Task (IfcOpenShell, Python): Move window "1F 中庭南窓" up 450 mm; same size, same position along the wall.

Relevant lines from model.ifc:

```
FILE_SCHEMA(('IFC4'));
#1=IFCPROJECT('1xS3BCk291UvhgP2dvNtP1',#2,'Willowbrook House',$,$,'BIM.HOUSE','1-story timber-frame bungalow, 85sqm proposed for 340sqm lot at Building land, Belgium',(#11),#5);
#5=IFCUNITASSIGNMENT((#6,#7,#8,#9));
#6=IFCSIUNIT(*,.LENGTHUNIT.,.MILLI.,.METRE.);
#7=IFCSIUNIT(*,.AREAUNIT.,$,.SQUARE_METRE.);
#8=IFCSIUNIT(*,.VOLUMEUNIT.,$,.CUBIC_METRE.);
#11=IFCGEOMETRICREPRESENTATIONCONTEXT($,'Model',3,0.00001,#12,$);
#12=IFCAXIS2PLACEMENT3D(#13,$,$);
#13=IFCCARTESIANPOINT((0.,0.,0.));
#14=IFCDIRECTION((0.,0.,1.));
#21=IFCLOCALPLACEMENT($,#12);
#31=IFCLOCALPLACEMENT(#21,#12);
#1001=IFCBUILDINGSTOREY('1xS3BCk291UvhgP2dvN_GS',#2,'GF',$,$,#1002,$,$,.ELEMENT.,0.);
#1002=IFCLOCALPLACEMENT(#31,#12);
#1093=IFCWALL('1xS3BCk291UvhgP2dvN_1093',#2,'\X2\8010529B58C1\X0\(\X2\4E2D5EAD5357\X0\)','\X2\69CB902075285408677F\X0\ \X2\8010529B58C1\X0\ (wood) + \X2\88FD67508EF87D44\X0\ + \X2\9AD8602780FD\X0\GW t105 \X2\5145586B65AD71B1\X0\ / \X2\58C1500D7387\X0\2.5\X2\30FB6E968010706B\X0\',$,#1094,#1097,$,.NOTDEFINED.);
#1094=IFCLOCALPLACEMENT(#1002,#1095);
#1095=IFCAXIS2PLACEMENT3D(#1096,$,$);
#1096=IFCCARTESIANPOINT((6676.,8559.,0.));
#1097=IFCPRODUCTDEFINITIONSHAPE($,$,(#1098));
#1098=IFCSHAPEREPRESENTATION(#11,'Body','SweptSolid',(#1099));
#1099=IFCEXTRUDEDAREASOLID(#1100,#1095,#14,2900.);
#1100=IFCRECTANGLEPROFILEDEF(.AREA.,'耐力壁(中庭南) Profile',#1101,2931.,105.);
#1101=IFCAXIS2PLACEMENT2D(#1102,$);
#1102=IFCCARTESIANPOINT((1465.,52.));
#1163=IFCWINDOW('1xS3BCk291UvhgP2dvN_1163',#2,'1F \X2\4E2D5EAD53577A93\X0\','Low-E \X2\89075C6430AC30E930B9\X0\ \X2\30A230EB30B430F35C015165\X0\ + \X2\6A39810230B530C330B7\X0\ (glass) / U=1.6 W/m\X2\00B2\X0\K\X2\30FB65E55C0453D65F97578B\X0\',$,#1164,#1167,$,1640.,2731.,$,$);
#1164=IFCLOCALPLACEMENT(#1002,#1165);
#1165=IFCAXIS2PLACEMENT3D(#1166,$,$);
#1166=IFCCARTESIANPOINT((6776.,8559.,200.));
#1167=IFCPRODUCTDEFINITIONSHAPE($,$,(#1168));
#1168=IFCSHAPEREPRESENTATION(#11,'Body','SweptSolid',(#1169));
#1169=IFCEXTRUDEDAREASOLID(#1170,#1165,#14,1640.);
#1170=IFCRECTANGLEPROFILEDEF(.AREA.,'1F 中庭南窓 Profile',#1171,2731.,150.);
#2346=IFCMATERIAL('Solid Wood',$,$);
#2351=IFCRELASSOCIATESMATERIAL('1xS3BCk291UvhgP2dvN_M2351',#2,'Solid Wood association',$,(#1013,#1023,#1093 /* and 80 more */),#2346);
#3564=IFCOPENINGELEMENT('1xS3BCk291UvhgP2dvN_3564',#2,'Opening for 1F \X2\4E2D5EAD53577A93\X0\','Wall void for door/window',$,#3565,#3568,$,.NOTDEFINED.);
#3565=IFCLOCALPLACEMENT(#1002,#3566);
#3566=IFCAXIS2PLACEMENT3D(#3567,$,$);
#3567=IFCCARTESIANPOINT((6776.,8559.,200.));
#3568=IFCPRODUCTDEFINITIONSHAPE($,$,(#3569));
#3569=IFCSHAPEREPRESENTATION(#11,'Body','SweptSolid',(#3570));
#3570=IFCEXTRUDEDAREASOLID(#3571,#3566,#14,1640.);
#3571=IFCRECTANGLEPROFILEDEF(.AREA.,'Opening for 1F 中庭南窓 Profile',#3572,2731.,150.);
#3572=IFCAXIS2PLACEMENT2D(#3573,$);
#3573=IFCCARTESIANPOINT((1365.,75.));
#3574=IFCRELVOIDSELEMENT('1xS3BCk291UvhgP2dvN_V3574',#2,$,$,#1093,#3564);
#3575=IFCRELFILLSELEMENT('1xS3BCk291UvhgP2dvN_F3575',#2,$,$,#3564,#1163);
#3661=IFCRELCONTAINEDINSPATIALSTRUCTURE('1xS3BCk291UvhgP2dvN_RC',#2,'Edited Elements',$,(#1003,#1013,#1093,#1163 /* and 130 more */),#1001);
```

```python
import numpy as np
import ifcopenshell
import ifcopenshell.api.geometry
import ifcopenshell.util.placement
import ifcopenshell.util.unit

model = ifcopenshell.open("model.ifc")
unit_scale = ifcopenshell.util.unit.calculate_unit_scale(model)

window = model.by_guid("1xS3BCk291UvhgP2dvN_1163")
opening = window.FillsVoids[0].RelatingOpeningElement
dz = 0.45 / unit_scale

shift = np.array([0.0, 0.0, dz])
# The window is not placed relative to its opening, so move both.
for product in (opening, window):
    matrix = ifcopenshell.util.placement.get_local_placement(product.ObjectPlacement)
    matrix[:3, 3] += shift
    ifcopenshell.api.geometry.edit_object_placement(model, product=product, matrix=matrix, is_si=False)

print(f"moved by {dz * unit_scale:+.3f} m")

model.write("model_v2.ifc")
```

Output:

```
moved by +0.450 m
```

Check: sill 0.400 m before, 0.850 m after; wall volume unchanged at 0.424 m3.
